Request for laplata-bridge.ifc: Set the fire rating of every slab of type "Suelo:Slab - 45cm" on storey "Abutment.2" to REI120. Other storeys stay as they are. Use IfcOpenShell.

First a look at what the model holds.

```python
import ifcopenshell
import ifcopenshell.util.element

model = ifcopenshell.open("laplata-bridge.ifc")
print(model.schema)
storey = next(s for s in model.by_type("IfcBuildingStorey") if s.Name == "Abutment.2")
slabs = [e for e in ifcopenshell.util.element.get_decomposition(storey) if e.is_a("IfcSlab")]
seen = {}
for e in slabs:
    element_type = ifcopenshell.util.element.get_type(e)
    key = (element_type.Name if element_type != e and element_type else None, ifcopenshell.util.element.get_pset(e, "Pset_SlabCommon", "FireRating"))
    seen[key] = seen.get(key, 0) + 1
for (name, value), count in sorted(seen.items(), key=str):
    print(count, "x", name, "|", value)
```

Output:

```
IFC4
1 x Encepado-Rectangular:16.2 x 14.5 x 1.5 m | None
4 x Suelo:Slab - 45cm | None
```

```python
import ifcopenshell
import ifcopenshell.api.pset
import ifcopenshell.util.element

model = ifcopenshell.open("laplata-bridge.ifc")

storey = next(s for s in model.by_type("IfcBuildingStorey") if s.Name == "Abutment.2")
slabs = [e for e in ifcopenshell.util.element.get_decomposition(storey) if e.is_a("IfcSlab")]

count = 0
for e in slabs:
    element_type = ifcopenshell.util.element.get_type(e)
    if element_type in (None, e) or element_type.Name != "Suelo:Slab - 45cm":
        continue
    # add_pset returns the element's existing set when there is one.
    pset = ifcopenshell.api.pset.add_pset(model, product=e, name="Pset_SlabCommon")
    ifcopenshell.api.pset.edit_pset(model, pset=pset, properties={"FireRating": "REI120"})
    count += 1

print(count, "slabs updated")

model.write("laplata-bridge_edited.ifc")
```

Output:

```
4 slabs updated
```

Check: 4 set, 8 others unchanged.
